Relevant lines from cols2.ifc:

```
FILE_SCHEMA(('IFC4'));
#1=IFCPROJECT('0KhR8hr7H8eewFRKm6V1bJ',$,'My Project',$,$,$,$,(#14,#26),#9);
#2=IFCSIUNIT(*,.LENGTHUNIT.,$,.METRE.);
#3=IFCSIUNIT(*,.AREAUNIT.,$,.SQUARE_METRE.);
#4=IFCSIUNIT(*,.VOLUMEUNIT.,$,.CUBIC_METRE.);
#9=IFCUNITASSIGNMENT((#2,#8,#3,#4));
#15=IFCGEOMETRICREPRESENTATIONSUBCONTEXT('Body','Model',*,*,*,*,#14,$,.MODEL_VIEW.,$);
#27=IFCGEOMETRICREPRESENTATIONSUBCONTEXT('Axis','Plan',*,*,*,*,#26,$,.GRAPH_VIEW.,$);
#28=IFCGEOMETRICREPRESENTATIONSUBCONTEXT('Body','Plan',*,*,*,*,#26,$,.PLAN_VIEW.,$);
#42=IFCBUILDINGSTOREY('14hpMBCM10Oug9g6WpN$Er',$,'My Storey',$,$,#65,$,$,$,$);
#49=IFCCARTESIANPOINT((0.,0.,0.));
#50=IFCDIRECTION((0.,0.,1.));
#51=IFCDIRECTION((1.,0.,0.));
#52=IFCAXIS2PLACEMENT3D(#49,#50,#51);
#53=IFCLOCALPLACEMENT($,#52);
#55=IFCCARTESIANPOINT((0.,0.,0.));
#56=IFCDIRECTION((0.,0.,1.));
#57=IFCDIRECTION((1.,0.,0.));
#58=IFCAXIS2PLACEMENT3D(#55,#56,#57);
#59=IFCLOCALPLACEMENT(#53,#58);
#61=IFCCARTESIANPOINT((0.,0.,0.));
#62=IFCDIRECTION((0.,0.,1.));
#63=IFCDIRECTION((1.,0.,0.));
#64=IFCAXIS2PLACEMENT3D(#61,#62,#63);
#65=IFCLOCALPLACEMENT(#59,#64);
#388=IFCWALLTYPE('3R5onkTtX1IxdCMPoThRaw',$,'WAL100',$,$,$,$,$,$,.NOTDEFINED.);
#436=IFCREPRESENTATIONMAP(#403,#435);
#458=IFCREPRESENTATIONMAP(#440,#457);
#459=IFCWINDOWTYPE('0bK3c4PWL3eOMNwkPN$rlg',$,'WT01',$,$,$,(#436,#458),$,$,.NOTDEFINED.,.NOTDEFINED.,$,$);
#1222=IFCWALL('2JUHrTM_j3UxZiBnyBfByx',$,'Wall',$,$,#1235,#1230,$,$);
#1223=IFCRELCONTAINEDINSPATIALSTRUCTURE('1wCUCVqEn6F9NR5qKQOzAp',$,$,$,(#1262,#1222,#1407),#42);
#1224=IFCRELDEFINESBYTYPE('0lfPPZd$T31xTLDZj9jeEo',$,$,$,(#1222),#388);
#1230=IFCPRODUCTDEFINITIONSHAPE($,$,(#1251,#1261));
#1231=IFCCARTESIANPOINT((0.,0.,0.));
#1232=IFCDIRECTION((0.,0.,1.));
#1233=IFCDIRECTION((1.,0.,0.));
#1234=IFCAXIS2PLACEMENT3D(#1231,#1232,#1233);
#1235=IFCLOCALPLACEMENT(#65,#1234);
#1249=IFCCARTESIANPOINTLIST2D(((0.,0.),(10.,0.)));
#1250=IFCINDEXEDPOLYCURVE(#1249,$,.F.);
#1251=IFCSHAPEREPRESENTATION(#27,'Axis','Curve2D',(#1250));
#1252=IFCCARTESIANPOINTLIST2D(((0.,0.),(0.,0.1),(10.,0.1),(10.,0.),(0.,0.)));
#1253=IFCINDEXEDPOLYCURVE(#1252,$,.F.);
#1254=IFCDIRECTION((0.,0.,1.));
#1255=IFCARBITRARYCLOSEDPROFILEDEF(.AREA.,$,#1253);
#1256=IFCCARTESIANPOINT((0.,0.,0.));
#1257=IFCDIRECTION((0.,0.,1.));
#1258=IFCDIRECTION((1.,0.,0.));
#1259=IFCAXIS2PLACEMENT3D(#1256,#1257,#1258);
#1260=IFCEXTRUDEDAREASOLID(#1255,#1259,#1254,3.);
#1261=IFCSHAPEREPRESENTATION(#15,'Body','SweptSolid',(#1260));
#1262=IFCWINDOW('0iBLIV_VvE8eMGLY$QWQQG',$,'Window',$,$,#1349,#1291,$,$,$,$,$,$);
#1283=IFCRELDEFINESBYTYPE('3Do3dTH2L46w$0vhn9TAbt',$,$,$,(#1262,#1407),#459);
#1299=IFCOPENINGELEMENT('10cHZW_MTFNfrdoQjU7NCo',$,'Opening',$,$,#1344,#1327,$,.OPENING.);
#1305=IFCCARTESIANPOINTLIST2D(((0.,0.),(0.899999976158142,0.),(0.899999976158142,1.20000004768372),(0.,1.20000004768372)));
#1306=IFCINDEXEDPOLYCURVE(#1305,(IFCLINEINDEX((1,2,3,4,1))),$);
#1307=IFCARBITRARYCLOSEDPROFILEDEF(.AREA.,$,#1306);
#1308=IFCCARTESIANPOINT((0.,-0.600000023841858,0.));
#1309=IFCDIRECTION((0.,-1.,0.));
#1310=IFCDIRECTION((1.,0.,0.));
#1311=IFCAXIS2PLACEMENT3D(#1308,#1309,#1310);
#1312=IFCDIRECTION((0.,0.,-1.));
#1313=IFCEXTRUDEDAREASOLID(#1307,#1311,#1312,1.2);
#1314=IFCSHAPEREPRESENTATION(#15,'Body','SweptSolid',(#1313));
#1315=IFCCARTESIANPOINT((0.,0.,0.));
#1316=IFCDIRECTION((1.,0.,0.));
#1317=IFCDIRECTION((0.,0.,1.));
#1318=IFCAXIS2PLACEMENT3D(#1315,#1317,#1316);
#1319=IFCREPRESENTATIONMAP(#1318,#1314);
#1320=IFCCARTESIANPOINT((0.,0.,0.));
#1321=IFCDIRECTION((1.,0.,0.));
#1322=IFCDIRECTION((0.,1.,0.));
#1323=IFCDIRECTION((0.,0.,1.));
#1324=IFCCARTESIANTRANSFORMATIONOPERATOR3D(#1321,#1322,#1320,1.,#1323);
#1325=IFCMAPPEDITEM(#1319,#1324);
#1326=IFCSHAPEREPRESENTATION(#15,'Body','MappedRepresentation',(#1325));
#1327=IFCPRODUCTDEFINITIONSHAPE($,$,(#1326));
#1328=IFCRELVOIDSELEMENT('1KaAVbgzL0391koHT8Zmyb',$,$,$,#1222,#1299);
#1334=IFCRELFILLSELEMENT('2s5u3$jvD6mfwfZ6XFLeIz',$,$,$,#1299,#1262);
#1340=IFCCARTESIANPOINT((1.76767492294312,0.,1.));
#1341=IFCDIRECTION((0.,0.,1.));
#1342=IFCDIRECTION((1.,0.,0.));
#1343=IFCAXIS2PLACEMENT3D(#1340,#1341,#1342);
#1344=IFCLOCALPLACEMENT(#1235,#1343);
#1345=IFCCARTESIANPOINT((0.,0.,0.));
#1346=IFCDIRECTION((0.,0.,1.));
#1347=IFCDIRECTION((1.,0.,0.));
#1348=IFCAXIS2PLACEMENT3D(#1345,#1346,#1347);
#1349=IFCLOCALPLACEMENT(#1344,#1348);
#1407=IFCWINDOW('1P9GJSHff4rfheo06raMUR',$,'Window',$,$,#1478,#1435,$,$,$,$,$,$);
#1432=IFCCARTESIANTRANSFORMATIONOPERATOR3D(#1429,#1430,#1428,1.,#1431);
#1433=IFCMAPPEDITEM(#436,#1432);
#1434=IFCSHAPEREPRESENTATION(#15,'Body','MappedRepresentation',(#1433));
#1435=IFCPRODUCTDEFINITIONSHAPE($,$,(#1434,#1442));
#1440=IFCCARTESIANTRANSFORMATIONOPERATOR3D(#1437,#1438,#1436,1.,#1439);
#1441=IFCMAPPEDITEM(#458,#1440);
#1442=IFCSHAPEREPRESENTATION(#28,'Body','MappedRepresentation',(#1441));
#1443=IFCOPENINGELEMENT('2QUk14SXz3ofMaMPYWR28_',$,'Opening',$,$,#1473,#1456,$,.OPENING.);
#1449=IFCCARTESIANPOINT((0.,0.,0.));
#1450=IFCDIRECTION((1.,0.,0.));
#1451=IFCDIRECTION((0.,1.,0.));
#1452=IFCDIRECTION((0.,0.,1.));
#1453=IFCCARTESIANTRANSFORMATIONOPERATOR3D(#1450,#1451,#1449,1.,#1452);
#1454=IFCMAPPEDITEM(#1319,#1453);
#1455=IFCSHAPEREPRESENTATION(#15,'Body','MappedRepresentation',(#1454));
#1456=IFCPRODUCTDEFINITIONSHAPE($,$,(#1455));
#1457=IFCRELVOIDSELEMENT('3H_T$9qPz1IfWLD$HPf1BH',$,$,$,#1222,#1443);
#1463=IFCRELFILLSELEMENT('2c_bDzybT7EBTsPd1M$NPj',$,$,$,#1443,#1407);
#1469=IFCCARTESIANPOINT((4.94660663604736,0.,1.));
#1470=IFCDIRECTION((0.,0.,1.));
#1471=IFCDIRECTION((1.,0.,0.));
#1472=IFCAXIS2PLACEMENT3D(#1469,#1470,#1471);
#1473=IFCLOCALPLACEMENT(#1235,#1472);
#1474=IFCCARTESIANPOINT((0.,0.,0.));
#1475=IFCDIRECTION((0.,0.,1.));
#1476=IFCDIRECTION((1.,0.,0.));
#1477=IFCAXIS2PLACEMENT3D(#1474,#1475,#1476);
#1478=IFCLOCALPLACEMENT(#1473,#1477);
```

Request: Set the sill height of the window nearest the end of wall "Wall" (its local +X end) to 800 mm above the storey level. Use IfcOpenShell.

```python
import numpy as np
import ifcopenshell
import ifcopenshell.api.geometry
import ifcopenshell.geom
import ifcopenshell.util.element
import ifcopenshell.util.placement
import ifcopenshell.util.shape
import ifcopenshell.util.unit

model = ifcopenshell.open("cols2.ifc")
unit_scale = ifcopenshell.util.unit.calculate_unit_scale(model)

window = model.by_guid("1P9GJSHff4rfheo06raMUR")
opening = window.FillsVoids[0].RelatingOpeningElement
storey = ifcopenshell.util.element.get_container(window, ifc_class="IfcBuildingStorey")
level = ifcopenshell.util.placement.get_local_placement(storey.ObjectPlacement)[2, 3]

# The opening's origin need not be at the sill, so measure its lowest point.
shape = ifcopenshell.geom.create_shape(ifcopenshell.geom.settings(), opening)
bottom = ifcopenshell.util.shape.get_shape_bottom_elevation(shape, shape.geometry) / unit_scale
dz = level + 0.8 - bottom

shift = np.array([0.0, 0.0, dz])
# The window is placed relative to its opening, so it follows when the opening moves.
matrix = ifcopenshell.util.placement.get_local_placement(opening.ObjectPlacement)
matrix[:3, 3] += shift
ifcopenshell.api.geometry.edit_object_placement(
    model, product=opening, matrix=matrix, is_si=False, should_transform_children=True
)

print(f"moved by {dz * unit_scale:+.3f} m")

model.write("cols2_updated.ifc")
```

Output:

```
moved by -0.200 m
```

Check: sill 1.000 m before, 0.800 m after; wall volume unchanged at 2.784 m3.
